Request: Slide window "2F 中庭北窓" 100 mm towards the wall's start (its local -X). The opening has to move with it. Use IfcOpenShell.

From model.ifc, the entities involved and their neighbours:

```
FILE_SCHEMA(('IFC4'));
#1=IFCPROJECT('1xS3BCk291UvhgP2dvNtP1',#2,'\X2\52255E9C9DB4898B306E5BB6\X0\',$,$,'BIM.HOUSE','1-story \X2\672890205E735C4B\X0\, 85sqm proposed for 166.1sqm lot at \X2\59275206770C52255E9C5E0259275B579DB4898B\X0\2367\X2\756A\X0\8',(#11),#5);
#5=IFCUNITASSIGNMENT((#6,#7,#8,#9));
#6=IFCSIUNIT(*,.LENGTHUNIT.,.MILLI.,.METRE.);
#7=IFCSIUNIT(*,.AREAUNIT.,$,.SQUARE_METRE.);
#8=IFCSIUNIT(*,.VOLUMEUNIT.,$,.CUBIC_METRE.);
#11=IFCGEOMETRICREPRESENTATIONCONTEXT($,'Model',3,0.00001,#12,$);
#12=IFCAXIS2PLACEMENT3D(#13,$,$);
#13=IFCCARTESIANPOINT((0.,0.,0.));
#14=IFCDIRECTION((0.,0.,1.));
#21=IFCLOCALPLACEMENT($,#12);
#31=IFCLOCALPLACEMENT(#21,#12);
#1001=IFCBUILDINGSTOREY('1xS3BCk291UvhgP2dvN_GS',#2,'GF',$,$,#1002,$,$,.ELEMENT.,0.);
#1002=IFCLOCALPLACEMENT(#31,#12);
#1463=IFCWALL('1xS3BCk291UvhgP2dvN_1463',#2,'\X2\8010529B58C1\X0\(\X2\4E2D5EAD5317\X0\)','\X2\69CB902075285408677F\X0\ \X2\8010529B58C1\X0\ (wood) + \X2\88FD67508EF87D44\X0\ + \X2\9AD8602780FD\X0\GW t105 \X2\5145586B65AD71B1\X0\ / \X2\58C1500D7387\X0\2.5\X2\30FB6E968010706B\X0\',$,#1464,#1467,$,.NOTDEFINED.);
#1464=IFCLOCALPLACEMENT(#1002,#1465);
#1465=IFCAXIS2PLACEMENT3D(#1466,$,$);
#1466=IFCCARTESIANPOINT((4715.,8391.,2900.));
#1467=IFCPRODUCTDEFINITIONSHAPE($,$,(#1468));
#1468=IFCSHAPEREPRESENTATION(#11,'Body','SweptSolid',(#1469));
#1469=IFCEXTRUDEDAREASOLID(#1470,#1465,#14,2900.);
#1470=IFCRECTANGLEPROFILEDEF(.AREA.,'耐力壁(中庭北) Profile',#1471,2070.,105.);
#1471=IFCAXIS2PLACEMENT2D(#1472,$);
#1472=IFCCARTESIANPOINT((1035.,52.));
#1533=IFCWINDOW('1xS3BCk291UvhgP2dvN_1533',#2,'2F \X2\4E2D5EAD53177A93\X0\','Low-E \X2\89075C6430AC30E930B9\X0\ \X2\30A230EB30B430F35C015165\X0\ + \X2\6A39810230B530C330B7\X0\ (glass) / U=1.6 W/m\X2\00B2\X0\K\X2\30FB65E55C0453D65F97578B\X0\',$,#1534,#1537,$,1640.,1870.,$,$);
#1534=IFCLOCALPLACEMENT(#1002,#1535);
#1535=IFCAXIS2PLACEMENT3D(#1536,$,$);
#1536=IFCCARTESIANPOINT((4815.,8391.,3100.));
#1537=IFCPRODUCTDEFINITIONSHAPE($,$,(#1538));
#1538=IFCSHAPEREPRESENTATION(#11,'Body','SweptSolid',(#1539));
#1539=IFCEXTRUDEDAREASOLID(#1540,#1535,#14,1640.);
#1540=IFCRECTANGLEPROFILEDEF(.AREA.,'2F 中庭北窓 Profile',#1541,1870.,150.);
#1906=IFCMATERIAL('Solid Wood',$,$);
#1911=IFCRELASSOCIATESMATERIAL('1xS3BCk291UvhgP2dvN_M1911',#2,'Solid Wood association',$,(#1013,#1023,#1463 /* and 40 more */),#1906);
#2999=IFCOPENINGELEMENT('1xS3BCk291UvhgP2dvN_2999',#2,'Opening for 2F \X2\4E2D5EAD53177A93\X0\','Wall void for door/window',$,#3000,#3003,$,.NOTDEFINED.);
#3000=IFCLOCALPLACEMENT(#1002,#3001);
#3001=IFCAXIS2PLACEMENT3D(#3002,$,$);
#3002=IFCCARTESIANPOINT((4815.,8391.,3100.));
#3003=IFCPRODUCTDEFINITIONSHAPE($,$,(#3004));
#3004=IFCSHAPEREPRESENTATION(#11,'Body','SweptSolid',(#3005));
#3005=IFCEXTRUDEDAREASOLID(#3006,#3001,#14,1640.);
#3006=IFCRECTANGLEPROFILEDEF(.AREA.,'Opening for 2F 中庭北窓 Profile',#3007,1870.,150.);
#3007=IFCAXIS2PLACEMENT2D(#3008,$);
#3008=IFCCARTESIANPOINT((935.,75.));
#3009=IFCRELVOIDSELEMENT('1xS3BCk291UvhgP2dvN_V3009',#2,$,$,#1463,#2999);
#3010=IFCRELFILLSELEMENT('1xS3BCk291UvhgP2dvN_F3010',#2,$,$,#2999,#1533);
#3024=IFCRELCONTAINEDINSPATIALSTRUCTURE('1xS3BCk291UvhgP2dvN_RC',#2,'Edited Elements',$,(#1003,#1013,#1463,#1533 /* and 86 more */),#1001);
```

```python
import ifcopenshell
import ifcopenshell.api.geometry
import ifcopenshell.util.placement

model = ifcopenshell.open("model.ifc")

window = model.by_id(1533)
opening = window.FillsVoids[0].RelatingOpeningElement
wall = opening.VoidsElements[0].RelatingBuildingElement

wall_matrix = ifcopenshell.util.placement.get_local_placement(wall.ObjectPlacement)
shift = wall_matrix[:3, 0] * -100.0
before = ifcopenshell.util.placement.get_local_placement(window.ObjectPlacement)[:3, 3].copy()

# The window is not placed relative to its opening, so move both.
for product in (opening, window):
    matrix = ifcopenshell.util.placement.get_local_placement(product.ObjectPlacement)
    matrix[:3, 3] += shift
    ifcopenshell.api.geometry.edit_object_placement(model, product=product, matrix=matrix, is_si=False)

after = ifcopenshell.util.placement.get_local_placement(window.ObjectPlacement)[:3, 3]
print("window moved by", (after - before).round(3) + 0.0)

model.write("model_edited.ifc")
```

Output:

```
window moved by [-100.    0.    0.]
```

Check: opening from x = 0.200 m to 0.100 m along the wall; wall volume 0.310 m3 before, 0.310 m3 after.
